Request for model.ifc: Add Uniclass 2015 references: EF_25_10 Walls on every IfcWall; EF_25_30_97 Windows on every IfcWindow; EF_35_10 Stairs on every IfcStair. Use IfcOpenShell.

First a look at what the model holds.

```python
import ifcopenshell

model = ifcopenshell.open("model.ifc")
print(model.schema)
print("classifications:", [c.Name for c in model.by_type("IfcClassification")])
for ifc_class in ("IfcDoor", "IfcRoof", "IfcStair", "IfcWall", "IfcWindow"):
    print(ifc_class, len(model.by_type(ifc_class)))
```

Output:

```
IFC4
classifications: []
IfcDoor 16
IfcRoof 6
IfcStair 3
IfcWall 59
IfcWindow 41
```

```python
import ifcopenshell
import ifcopenshell.api.classification

model = ifcopenshell.open("model.ifc")

system = ifcopenshell.api.classification.add_classification(model, classification="Uniclass 2015")

codes = {
    "IfcWall": ("EF_25_10", "Walls"),
    "IfcWindow": ("EF_25_30_97", "Windows"),
    "IfcStair": ("EF_35_10", "Stairs"),
}
for ifc_class, (code, name) in codes.items():
    products = model.by_type(ifc_class)
    ifcopenshell.api.classification.add_reference(
        model, products=products, classification=system, identification=code, name=name
    )
    print(code, len(products))

model.write("model_edited.ifc")
```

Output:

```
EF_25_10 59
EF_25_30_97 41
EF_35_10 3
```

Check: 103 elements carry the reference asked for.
